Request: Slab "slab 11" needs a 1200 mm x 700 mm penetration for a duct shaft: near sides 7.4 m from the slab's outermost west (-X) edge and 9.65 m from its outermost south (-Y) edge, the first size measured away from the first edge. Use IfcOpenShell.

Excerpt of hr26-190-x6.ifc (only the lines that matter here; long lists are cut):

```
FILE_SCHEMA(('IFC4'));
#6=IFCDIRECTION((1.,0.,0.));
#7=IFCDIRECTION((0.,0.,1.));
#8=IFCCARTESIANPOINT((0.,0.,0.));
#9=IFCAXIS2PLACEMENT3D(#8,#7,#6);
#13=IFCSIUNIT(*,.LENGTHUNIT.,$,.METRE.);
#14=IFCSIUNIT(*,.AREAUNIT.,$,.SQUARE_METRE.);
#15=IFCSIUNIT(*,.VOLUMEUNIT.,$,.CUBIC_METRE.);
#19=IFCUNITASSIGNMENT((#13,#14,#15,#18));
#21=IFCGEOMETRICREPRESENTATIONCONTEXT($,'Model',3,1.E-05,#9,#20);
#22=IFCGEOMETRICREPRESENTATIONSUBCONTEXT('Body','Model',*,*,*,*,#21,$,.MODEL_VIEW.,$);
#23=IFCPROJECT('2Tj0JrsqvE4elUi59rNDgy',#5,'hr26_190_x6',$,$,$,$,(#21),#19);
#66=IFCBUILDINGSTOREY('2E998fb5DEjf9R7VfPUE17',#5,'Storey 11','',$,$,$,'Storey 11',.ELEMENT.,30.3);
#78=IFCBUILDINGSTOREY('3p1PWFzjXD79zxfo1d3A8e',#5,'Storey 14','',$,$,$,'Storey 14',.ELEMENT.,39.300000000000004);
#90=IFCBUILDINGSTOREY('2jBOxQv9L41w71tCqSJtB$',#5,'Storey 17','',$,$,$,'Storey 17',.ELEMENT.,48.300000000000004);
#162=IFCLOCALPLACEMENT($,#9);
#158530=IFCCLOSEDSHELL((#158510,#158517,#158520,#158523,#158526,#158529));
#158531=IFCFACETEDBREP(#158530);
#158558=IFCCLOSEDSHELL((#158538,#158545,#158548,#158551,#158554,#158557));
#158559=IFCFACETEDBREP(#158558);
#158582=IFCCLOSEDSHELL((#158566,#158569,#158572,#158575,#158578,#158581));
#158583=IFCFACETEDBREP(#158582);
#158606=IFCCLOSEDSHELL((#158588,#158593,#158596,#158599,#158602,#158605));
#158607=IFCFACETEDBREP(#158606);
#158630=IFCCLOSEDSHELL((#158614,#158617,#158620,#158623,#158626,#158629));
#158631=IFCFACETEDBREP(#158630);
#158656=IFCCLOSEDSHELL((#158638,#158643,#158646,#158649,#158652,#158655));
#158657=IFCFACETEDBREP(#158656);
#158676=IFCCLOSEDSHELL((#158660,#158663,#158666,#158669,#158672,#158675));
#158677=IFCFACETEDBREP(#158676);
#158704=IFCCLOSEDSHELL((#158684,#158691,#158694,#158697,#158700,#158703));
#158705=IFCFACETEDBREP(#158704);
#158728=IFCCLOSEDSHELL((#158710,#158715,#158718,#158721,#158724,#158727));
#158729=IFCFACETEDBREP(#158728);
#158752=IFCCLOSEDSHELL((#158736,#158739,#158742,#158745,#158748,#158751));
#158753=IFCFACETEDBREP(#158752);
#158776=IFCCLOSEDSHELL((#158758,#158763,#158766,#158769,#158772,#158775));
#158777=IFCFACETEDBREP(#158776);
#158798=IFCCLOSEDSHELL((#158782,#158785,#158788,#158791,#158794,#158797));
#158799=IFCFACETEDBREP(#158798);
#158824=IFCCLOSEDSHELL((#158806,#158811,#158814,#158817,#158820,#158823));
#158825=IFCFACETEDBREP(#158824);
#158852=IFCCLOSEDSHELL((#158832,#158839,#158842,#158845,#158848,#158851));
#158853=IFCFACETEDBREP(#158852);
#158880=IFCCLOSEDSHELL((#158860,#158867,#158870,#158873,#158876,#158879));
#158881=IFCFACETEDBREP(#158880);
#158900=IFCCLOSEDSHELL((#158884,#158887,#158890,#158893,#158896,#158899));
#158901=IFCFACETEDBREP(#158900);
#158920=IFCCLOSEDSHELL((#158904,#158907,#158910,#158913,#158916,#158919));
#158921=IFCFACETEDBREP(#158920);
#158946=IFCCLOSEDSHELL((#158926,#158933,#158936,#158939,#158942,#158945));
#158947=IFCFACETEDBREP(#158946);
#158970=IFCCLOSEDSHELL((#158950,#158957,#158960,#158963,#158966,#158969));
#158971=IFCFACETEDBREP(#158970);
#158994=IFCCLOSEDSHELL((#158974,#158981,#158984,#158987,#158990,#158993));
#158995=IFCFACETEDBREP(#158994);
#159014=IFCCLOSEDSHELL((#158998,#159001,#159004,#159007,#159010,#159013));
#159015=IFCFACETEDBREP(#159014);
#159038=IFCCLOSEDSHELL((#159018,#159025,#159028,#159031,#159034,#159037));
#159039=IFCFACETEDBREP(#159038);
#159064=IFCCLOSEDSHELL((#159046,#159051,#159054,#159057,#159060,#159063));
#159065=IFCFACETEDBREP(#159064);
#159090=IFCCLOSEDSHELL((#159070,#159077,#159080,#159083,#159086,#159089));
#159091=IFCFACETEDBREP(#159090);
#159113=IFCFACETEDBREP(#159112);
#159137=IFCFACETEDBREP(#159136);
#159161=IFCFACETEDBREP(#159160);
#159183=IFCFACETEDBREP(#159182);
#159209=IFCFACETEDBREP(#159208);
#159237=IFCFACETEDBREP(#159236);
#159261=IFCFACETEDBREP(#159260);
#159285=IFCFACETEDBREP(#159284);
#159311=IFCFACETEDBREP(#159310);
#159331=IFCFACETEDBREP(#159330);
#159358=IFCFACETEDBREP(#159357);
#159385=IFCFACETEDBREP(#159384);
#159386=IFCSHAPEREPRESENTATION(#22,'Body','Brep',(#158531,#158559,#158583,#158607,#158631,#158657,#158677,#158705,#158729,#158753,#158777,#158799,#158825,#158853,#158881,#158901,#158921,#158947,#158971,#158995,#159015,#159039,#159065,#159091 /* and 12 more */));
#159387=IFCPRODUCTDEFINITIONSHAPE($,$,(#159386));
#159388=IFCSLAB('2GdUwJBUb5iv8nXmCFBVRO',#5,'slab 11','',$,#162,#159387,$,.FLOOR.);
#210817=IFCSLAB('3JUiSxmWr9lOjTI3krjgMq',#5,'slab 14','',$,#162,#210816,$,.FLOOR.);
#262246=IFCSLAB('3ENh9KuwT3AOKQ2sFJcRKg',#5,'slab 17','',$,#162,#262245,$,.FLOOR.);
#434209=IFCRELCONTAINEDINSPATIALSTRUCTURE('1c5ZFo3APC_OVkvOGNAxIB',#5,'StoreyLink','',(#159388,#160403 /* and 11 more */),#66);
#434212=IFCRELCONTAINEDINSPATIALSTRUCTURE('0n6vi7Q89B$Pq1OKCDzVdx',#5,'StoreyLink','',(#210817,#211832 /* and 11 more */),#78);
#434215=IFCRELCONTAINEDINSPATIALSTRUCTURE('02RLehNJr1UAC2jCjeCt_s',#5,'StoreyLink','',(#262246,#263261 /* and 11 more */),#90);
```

```python
import numpy as np
import ifcopenshell
import ifcopenshell.api.feature
import ifcopenshell.api.geometry
import ifcopenshell.api.root
import ifcopenshell.geom
import ifcopenshell.util.placement
import ifcopenshell.util.representation
import ifcopenshell.util.shape
import ifcopenshell.util.unit

model = ifcopenshell.open("hr26-190-x6.ifc")
unit_scale = ifcopenshell.util.unit.calculate_unit_scale(model)
settings = ifcopenshell.geom.settings()


def volume(element):
    """Net volume in cubic metres, openings subtracted."""
    shape = ifcopenshell.geom.create_shape(settings, element)
    return ifcopenshell.util.shape.get_volume(shape.geometry)


slab = model.by_guid("2GdUwJBUb5iv8nXmCFBVRO")
before = volume(slab)

# Extent in the slab's own axes, in metres. The edges named are its -X and -Y sides.
slab_shape = ifcopenshell.geom.create_shape(settings, slab)
vertices = ifcopenshell.util.shape.get_vertices(slab_shape.geometry)
x_min, y_min, bottom = vertices.min(axis=0)
top = vertices[:, 2].max()

opening = ifcopenshell.api.root.create_entity(model, ifc_class="IfcOpeningElement", name="Duct shaft opening", predefined_type="OPENING")
context = ifcopenshell.util.representation.get_context(model, "Model", "Body", "MODEL_VIEW")
width, depth = 1.2, 0.7
outline = [(0.0, 0.0), (width, 0.0), (width, depth), (0.0, depth), (0.0, 0.0)]
# Overshoot both faces by 50 mm so the cut is clean.
shape = ifcopenshell.api.geometry.add_slab_representation(
    model, context=context, depth=top - bottom + 0.1, polyline=outline
)
ifcopenshell.api.geometry.assign_representation(model, product=opening, representation=shape)

matrix = ifcopenshell.util.placement.get_local_placement(slab.ObjectPlacement)
matrix[:, 3] = matrix @ np.append(np.array([x_min + 7.4, y_min + 9.65, bottom - 0.05]) / unit_scale, 1.0)
ifcopenshell.api.geometry.edit_object_placement(model, product=opening, matrix=matrix, is_si=False)
ifcopenshell.api.feature.add_feature(model, feature=opening, element=slab)

after = volume(slab)

print(f"slab volume {before:.3f} -> {after:.3f} m3")

model.write("hr26-190-x6-out.ifc")
```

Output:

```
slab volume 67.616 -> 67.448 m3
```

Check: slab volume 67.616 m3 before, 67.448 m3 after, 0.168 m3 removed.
